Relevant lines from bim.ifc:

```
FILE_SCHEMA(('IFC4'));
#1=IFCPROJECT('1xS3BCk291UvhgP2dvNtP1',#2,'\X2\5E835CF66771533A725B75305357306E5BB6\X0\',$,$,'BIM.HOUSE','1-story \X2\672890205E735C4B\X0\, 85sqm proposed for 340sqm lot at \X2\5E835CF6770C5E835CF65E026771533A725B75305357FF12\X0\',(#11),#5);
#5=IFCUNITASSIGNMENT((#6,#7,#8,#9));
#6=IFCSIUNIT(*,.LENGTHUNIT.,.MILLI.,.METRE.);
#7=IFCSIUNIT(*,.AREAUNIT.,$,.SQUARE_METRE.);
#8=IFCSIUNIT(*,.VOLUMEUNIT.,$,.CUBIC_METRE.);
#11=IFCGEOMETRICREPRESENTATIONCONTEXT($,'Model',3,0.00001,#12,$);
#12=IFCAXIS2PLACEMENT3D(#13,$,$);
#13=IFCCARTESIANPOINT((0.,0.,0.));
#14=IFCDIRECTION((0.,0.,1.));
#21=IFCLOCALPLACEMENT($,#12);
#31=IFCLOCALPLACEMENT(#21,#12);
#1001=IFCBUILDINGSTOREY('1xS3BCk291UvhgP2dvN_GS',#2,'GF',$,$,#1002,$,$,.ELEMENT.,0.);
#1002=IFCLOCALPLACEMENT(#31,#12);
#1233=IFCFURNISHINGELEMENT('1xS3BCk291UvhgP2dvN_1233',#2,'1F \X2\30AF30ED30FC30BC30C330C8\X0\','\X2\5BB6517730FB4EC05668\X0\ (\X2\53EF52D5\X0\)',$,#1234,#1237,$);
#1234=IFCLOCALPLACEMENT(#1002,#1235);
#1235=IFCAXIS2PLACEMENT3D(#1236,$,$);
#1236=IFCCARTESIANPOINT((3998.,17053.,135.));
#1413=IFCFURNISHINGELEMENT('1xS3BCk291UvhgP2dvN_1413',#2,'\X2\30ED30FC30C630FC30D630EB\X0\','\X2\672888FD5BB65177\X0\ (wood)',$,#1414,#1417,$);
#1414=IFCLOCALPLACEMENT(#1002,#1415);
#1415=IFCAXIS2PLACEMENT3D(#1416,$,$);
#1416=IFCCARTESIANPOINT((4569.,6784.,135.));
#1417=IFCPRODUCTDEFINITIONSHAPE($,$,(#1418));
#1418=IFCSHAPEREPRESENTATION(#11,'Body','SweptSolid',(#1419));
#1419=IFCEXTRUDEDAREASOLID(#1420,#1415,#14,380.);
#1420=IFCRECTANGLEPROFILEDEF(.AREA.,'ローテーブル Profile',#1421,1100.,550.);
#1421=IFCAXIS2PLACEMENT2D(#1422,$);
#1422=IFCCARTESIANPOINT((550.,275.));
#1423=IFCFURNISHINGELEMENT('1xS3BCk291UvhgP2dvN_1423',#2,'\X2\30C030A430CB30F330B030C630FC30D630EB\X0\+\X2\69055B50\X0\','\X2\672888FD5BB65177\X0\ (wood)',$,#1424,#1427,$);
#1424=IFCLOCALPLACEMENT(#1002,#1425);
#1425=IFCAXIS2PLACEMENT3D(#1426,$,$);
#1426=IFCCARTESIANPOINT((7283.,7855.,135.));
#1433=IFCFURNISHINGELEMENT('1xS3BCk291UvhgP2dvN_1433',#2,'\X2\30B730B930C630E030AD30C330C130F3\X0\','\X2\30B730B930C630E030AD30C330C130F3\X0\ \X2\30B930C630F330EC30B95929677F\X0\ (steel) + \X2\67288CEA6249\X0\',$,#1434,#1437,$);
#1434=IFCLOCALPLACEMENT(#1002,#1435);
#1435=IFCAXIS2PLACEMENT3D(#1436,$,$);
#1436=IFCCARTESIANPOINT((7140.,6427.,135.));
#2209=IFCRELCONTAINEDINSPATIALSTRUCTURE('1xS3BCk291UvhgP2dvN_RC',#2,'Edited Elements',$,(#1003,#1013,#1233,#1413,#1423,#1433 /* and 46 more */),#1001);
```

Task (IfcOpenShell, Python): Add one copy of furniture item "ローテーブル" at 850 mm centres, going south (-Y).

```python
import numpy as np
import ifcopenshell
import ifcopenshell.api.geometry
import ifcopenshell.api.root
import ifcopenshell.util.element
import ifcopenshell.util.placement
import ifcopenshell.util.unit

model = ifcopenshell.open("bim.ifc")
unit_scale = ifcopenshell.util.unit.calculate_unit_scale(model)


def reuse_history(source, copy):
    """copy_class also copies each property set's owner history, people and application; keep the originals."""
    for rel in copy.IsDefinedBy:
        if rel.is_a("IfcRelDefinesByProperties") and (history := rel.RelatingPropertyDefinition.OwnerHistory):
            rel.RelatingPropertyDefinition.OwnerHistory = source.OwnerHistory
            ifcopenshell.util.element.remove_deep2(model, history)


source = model.by_id(1413)
base = ifcopenshell.util.placement.get_local_placement(source.ObjectPlacement)
step = np.array([0.0, -1.0, 0.0]) * 0.85 / unit_scale

for i in range(1, 2):
    copy = ifcopenshell.api.root.copy_class(model, product=source)
    copy.Representation = ifcopenshell.util.element.copy_deep(
        model, source.Representation, exclude=["IfcGeometricRepresentationContext", "IfcRepresentationMap"]
    )
    reuse_history(source, copy)
    matrix = base.copy()
    matrix[:3, 3] += i * step
    print("added at", matrix[:3, 3].round(3) + 0.0)
    ifcopenshell.api.geometry.edit_object_placement(model, product=copy, matrix=matrix, is_si=False)

model.write("bim_v2.ifc")
```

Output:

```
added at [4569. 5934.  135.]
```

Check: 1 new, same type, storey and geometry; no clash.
